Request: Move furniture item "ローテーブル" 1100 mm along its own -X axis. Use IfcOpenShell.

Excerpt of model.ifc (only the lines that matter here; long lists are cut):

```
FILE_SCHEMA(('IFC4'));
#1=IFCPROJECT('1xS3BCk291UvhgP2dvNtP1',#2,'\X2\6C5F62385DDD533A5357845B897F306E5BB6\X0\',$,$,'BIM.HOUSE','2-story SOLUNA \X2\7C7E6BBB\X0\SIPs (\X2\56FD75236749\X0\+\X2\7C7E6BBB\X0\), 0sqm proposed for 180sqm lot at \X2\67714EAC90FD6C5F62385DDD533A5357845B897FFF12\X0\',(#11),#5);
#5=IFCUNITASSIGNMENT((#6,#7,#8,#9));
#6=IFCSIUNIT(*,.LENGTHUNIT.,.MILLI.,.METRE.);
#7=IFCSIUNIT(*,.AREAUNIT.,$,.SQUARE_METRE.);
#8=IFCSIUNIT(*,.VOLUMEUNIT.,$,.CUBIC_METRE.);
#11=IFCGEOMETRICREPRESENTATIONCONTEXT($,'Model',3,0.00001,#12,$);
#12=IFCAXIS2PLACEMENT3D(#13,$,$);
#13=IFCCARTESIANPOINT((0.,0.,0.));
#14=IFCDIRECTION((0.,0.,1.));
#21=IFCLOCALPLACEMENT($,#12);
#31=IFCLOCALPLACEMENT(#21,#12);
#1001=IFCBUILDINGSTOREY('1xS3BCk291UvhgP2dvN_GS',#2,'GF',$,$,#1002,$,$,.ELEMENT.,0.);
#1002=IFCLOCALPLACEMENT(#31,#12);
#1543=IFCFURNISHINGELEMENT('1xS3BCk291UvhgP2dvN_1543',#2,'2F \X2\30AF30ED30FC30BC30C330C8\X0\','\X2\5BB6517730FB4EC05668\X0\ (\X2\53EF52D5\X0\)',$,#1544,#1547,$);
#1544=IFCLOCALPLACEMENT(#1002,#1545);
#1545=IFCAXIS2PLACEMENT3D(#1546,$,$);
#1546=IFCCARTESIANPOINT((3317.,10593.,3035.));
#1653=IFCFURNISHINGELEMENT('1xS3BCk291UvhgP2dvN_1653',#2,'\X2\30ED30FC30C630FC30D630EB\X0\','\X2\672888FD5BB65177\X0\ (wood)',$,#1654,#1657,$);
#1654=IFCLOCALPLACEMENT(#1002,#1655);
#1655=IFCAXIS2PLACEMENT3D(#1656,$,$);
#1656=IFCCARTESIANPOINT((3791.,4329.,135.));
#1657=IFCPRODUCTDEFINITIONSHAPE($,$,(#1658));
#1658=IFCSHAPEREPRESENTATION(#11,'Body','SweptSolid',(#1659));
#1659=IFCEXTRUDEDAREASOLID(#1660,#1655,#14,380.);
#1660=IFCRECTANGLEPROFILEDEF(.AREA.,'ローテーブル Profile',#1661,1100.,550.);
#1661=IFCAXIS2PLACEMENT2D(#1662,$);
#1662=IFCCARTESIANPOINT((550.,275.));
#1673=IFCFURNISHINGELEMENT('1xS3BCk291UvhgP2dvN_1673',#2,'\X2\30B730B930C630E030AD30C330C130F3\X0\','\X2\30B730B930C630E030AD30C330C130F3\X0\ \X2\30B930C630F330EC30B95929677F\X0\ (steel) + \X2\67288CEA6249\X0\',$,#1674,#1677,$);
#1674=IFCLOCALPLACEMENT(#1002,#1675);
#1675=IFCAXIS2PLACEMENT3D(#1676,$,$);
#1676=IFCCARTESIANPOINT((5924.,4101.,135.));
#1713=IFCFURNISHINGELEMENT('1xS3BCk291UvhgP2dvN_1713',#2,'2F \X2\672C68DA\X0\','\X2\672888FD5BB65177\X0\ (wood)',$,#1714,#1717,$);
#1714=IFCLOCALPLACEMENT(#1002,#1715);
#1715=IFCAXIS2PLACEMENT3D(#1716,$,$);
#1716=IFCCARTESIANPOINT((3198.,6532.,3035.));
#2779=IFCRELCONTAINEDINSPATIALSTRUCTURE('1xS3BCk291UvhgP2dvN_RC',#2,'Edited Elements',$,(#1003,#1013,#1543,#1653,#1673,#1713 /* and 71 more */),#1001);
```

```python
import ifcopenshell
import ifcopenshell.api.geometry
import ifcopenshell.util.placement
import ifcopenshell.util.unit

model = ifcopenshell.open("model.ifc")
unit_scale = ifcopenshell.util.unit.calculate_unit_scale(model)

item = model.by_guid("1xS3BCk291UvhgP2dvN_1653")
matrix = ifcopenshell.util.placement.get_local_placement(item.ObjectPlacement)
matrix[:3, 3] -= matrix[:3, 0] * 1.1 / unit_scale
ifcopenshell.api.geometry.edit_object_placement(model, product=item, matrix=matrix, is_si=False)

print(ifcopenshell.util.placement.get_local_placement(item.ObjectPlacement).round(3) + 0.0)

model.write("model-out.ifc")
```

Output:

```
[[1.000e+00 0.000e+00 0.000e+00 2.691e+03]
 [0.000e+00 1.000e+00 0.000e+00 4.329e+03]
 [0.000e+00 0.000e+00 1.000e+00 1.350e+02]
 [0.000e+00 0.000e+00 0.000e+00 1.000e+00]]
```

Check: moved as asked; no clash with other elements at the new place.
